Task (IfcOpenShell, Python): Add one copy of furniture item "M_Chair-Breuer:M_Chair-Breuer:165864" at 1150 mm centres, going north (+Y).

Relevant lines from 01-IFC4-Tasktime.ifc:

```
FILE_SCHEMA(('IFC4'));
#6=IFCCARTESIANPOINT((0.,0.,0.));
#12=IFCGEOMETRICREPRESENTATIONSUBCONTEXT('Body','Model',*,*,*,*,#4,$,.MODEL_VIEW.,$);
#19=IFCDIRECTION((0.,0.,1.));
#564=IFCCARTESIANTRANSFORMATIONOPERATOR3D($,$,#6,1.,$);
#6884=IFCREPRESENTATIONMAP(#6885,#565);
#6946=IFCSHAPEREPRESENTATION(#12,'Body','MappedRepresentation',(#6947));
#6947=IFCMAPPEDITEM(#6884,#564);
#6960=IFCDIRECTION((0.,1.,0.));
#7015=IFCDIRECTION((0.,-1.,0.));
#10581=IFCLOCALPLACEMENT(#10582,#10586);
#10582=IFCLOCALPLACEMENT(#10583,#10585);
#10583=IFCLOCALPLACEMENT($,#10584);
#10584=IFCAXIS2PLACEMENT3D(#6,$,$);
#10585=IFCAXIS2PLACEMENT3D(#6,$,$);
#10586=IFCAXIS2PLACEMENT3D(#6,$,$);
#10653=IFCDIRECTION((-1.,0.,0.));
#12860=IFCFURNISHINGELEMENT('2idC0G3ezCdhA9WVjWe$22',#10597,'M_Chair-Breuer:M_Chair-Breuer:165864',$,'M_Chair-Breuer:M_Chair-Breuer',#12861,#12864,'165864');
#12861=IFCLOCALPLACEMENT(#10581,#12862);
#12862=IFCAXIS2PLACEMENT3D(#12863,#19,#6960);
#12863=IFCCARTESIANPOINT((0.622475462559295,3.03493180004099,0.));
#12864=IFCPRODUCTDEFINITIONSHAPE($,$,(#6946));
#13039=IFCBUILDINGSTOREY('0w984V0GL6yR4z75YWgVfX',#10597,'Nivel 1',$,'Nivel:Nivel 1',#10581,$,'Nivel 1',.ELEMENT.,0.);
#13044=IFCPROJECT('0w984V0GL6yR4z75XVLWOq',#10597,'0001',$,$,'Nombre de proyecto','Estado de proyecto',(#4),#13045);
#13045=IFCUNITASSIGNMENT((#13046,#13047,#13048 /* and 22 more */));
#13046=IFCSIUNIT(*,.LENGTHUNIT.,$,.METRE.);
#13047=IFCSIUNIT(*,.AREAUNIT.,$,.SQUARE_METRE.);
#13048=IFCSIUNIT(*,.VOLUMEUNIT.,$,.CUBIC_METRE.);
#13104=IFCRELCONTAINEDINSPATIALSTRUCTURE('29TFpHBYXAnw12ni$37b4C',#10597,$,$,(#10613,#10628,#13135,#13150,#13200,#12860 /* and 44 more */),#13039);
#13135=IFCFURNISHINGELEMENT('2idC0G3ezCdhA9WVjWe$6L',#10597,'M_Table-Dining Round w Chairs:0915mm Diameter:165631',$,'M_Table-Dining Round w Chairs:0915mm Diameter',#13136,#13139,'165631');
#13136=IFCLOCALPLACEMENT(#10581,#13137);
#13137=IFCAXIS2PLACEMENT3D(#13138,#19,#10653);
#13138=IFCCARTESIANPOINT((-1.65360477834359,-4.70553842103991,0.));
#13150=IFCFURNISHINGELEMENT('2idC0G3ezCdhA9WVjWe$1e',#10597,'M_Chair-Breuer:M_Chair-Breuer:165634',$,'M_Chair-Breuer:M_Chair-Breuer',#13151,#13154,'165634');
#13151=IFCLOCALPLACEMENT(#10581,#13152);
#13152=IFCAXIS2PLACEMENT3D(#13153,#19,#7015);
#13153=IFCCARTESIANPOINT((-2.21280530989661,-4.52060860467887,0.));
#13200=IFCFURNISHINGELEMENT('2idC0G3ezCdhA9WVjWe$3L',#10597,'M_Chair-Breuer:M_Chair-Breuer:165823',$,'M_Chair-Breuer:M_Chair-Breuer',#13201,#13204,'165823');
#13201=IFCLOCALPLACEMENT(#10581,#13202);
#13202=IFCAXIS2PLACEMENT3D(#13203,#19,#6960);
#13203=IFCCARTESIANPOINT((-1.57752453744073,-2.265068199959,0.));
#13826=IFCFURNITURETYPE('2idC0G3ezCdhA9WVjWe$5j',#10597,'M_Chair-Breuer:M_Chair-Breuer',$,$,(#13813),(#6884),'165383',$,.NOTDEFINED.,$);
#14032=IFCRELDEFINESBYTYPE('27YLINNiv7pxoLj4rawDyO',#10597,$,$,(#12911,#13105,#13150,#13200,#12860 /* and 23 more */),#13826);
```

```python
import numpy as np
import ifcopenshell
import ifcopenshell.api.geometry
import ifcopenshell.api.root
import ifcopenshell.util.element
import ifcopenshell.util.placement
import ifcopenshell.util.unit

model = ifcopenshell.open("01-IFC4-Tasktime.ifc")
unit_scale = ifcopenshell.util.unit.calculate_unit_scale(model)


def reuse_history(source, copy):
    """copy_class also copies each property set's owner history, people and application; keep the originals."""
    for rel in copy.IsDefinedBy:
        if rel.is_a("IfcRelDefinesByProperties") and (history := rel.RelatingPropertyDefinition.OwnerHistory):
            rel.RelatingPropertyDefinition.OwnerHistory = source.OwnerHistory
            ifcopenshell.util.element.remove_deep2(model, history)


source = model.by_guid("2idC0G3ezCdhA9WVjWe$22")
base = ifcopenshell.util.placement.get_local_placement(source.ObjectPlacement)
step = np.array([0.0, 1.0, 0.0]) * 1.15 / unit_scale

for i in range(1, 2):
    copy = ifcopenshell.api.root.copy_class(model, product=source)
    copy.Representation = ifcopenshell.util.element.copy_deep(
        model, source.Representation, exclude=["IfcGeometricRepresentationContext", "IfcRepresentationMap"]
    )
    copy.Name = "M_Chair-Breuer:M_Chair-Breuer"
    copy.Tag = None
    reuse_history(source, copy)
    matrix = base.copy()
    matrix[:3, 3] += i * step
    print("added at", matrix[:3, 3].round(3) + 0.0)
    ifcopenshell.api.geometry.edit_object_placement(model, product=copy, matrix=matrix, is_si=False)

model.write("01-IFC4-Tasktime-out.ifc")
```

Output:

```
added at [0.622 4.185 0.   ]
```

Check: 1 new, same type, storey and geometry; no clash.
